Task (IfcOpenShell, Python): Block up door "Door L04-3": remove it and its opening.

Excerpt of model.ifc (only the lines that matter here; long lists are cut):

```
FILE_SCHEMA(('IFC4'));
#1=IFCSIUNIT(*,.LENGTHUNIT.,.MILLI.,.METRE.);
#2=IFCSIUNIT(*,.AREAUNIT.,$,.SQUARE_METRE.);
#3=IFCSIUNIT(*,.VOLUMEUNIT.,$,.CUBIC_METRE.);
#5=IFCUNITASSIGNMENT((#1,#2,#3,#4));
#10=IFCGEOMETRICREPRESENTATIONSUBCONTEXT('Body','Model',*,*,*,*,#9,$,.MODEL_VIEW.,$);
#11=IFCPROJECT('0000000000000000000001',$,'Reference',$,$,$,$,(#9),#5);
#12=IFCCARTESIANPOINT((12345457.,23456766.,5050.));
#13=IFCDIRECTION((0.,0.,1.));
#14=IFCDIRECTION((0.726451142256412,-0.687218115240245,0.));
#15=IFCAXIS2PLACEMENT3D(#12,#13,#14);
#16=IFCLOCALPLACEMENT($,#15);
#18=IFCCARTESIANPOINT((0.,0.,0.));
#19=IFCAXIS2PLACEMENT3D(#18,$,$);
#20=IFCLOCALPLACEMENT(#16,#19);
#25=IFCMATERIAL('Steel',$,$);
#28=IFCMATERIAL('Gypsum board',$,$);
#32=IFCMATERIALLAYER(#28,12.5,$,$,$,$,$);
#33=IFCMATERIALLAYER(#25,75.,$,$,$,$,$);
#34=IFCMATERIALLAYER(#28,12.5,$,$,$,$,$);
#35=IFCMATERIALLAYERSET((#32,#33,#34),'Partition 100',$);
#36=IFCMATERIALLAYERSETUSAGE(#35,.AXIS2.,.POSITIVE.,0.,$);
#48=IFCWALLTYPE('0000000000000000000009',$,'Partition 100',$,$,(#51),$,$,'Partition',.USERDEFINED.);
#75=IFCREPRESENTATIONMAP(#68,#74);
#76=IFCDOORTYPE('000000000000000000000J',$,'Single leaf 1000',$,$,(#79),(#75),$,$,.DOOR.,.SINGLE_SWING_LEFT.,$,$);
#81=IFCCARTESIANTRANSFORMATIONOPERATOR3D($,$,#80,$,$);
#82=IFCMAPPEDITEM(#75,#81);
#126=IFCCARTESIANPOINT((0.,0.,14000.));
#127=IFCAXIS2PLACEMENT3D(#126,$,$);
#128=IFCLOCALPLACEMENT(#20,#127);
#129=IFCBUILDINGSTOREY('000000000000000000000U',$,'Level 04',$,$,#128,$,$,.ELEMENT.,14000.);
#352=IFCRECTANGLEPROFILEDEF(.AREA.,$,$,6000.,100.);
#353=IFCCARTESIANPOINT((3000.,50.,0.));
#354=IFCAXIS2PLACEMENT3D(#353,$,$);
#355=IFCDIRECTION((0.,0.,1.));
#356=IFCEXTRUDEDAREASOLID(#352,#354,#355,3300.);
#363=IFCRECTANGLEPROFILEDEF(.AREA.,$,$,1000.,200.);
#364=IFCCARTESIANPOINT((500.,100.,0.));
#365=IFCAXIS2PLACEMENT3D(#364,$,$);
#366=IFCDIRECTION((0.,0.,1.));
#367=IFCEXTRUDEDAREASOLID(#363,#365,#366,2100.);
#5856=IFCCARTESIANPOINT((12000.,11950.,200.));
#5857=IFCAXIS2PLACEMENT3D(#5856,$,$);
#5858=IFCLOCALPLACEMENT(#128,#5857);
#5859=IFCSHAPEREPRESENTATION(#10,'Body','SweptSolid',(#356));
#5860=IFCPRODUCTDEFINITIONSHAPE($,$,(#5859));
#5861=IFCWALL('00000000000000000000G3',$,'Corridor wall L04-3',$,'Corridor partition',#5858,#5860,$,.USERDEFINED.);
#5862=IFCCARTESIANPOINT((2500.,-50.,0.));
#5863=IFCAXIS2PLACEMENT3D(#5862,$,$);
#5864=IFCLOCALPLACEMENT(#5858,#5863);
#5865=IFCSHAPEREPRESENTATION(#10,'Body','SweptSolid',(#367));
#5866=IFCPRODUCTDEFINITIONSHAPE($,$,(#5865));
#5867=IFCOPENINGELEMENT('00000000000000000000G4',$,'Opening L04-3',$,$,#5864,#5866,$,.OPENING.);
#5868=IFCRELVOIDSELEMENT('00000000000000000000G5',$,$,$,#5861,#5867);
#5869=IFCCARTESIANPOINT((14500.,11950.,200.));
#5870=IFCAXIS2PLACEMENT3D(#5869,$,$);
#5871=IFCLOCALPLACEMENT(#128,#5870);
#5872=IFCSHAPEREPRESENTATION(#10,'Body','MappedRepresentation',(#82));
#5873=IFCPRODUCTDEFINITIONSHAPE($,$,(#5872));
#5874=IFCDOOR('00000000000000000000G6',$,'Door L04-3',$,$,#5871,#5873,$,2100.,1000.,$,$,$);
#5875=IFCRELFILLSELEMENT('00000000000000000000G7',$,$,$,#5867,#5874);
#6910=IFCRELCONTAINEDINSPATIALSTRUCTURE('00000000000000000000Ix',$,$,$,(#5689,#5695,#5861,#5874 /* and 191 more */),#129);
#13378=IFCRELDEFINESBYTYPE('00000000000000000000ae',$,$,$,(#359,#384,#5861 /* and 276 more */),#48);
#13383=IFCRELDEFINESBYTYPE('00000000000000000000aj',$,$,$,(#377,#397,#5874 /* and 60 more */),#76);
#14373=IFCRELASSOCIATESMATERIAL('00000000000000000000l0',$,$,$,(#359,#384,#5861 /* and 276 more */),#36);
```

```python
import ifcopenshell
import ifcopenshell.api.feature
import ifcopenshell.api.root
import ifcopenshell.geom
import ifcopenshell.util.shape

model = ifcopenshell.open("model.ifc")
settings = ifcopenshell.geom.settings()


def volume(element):
    """Net volume in cubic metres, openings subtracted."""
    shape = ifcopenshell.geom.create_shape(settings, element)
    return ifcopenshell.util.shape.get_volume(shape.geometry)


door = model.by_guid("00000000000000000000G6")
opening = door.FillsVoids[0].RelatingOpeningElement
wall = opening.VoidsElements[0].RelatingBuildingElement
before = volume(wall)

ifcopenshell.api.root.remove_product(model, product=door)
ifcopenshell.api.feature.remove_feature(model, feature=opening)

after = volume(wall)

print(f"wall volume {before:.3f} -> {after:.3f} m3")

model.write("model-out.ifc")
```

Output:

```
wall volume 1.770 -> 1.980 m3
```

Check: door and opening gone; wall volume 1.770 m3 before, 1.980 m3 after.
